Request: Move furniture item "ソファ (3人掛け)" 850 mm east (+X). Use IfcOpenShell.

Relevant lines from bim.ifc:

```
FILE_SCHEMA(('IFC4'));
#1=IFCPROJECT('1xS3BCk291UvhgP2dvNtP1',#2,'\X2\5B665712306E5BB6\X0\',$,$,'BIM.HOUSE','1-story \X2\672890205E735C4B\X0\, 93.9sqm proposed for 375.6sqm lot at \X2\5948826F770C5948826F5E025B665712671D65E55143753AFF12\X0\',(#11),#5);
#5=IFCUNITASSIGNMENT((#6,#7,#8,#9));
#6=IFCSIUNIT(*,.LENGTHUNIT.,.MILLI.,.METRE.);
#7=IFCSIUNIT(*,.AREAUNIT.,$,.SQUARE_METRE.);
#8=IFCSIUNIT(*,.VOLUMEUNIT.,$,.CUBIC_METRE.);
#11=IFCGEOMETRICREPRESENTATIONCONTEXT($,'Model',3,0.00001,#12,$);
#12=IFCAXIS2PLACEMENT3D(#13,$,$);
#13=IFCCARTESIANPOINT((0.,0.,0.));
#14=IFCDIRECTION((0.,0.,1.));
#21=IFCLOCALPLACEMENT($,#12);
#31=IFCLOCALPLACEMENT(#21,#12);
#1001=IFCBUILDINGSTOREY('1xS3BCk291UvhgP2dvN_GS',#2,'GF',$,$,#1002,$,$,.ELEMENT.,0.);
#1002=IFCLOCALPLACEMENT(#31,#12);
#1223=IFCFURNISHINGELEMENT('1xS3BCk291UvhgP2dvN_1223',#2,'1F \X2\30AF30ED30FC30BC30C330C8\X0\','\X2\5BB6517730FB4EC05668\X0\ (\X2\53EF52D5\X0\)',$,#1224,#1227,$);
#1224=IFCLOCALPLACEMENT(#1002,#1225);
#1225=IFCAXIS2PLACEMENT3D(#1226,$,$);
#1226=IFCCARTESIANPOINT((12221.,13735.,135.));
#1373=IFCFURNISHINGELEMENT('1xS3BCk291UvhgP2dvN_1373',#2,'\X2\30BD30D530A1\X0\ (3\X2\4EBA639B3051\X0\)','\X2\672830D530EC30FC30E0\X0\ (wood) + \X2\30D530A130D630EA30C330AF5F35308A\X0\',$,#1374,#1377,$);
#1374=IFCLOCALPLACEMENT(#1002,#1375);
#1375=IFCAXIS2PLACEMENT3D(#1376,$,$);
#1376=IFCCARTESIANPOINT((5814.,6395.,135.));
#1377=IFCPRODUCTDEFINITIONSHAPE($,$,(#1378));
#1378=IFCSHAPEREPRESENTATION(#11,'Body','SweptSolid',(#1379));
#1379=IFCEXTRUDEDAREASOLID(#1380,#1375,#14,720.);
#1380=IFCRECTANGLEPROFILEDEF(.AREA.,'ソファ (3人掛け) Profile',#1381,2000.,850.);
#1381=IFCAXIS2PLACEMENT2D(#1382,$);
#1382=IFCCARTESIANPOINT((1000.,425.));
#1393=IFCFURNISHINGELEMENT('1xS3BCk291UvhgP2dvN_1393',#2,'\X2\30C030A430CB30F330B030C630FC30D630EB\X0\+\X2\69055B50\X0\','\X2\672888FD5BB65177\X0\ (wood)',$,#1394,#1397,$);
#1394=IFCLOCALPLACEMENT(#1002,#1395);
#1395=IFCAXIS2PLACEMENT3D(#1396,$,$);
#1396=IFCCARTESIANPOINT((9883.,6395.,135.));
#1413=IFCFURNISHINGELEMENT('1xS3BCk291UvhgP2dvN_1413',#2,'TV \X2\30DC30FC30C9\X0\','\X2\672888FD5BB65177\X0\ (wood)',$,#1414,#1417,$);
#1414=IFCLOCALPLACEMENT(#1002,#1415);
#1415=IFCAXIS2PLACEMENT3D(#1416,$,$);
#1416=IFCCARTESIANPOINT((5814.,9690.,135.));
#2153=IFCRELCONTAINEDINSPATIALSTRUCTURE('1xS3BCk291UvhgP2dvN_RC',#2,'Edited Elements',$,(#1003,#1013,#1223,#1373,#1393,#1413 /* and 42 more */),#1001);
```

```python
import ifcopenshell
import ifcopenshell.api.geometry
import ifcopenshell.util.placement
import ifcopenshell.util.unit

model = ifcopenshell.open("bim.ifc")
unit_scale = ifcopenshell.util.unit.calculate_unit_scale(model)

item = model.by_guid("1xS3BCk291UvhgP2dvN_1373")
matrix = ifcopenshell.util.placement.get_local_placement(item.ObjectPlacement)
matrix[0, 3] += 0.85 / unit_scale
ifcopenshell.api.geometry.edit_object_placement(model, product=item, matrix=matrix, is_si=False)

print(ifcopenshell.util.placement.get_local_placement(item.ObjectPlacement).round(3) + 0.0)

model.write("bim_rev.ifc")
```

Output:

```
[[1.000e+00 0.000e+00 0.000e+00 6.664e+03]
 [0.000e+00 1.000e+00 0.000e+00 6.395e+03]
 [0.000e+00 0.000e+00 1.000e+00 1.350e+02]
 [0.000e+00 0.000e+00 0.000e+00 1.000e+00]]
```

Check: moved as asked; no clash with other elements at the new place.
